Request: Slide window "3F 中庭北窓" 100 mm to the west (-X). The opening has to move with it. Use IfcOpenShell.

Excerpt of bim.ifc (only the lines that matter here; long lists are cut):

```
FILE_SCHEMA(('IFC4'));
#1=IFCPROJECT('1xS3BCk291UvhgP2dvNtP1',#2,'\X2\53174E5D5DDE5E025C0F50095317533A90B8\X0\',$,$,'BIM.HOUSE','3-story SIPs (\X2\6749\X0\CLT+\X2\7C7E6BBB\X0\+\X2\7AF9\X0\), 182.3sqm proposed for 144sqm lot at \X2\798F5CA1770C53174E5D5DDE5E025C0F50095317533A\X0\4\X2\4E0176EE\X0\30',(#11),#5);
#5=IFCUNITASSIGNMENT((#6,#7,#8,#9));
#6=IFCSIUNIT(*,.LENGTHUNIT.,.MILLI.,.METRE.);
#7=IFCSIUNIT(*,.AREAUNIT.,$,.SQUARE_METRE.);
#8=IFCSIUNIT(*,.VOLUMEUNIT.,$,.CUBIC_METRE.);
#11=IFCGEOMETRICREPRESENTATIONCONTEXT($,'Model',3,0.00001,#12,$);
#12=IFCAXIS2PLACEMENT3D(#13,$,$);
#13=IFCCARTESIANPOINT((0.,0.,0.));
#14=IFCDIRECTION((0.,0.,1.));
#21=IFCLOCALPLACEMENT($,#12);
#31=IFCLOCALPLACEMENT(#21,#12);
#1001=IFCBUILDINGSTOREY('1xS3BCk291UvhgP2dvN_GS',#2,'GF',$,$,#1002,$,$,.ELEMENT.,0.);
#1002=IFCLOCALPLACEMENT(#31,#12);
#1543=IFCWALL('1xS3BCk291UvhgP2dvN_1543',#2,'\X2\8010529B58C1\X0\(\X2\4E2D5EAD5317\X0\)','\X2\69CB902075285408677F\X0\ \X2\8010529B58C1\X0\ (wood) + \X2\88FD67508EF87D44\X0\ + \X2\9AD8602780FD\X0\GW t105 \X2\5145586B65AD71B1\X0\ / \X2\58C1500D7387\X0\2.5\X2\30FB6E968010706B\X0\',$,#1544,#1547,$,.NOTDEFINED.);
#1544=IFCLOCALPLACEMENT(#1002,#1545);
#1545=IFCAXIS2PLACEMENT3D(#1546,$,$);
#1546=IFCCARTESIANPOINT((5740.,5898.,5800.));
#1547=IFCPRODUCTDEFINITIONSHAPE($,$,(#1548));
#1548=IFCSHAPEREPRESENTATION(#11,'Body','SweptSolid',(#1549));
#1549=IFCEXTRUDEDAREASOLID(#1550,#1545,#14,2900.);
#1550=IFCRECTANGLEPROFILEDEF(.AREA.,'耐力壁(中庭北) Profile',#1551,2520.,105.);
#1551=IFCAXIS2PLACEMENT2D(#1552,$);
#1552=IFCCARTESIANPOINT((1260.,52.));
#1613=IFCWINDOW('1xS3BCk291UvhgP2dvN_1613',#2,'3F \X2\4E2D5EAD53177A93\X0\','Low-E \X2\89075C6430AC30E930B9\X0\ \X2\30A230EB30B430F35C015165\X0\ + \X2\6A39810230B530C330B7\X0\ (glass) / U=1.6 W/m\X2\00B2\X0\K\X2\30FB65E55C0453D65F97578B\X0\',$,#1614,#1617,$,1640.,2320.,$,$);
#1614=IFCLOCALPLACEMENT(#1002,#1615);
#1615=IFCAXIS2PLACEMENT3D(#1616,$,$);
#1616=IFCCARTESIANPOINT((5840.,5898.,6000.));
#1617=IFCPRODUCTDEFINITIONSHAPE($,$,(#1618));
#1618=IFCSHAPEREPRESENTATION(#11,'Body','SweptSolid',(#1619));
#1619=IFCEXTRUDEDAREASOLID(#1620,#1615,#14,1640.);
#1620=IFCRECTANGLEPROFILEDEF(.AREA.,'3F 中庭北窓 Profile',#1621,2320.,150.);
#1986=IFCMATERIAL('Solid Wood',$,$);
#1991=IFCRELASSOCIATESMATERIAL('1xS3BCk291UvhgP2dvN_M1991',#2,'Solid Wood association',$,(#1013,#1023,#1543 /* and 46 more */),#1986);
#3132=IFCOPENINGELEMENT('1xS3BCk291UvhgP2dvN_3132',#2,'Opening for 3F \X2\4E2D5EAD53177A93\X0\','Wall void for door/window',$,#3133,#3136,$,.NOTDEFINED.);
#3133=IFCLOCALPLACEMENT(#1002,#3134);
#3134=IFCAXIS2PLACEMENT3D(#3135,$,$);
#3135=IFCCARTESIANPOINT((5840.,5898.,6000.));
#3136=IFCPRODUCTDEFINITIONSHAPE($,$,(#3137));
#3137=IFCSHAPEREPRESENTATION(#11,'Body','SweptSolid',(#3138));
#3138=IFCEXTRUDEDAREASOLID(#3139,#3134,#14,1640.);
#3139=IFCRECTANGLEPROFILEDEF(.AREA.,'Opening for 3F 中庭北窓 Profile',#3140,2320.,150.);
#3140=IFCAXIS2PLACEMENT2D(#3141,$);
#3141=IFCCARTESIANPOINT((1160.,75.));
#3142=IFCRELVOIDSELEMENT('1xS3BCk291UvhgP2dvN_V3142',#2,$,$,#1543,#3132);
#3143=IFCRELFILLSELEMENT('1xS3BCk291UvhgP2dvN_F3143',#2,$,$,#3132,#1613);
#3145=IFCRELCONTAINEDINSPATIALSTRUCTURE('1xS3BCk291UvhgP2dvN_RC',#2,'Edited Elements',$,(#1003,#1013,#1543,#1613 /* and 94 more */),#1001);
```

```python
import ifcopenshell
import ifcopenshell.api.geometry
import ifcopenshell.util.placement
import ifcopenshell.util.unit

model = ifcopenshell.open("bim.ifc")
unit_scale = ifcopenshell.util.unit.calculate_unit_scale(model)

window = model.by_guid("1xS3BCk291UvhgP2dvN_1613")
opening = window.FillsVoids[0].RelatingOpeningElement
wall = opening.VoidsElements[0].RelatingBuildingElement

wall_matrix = ifcopenshell.util.placement.get_local_placement(wall.ObjectPlacement)
shift = wall_matrix[:3, 0] * -0.1 / unit_scale
before = ifcopenshell.util.placement.get_local_placement(window.ObjectPlacement)[:3, 3].copy()

# The window is not placed relative to its opening, so move both.
for product in (opening, window):
    matrix = ifcopenshell.util.placement.get_local_placement(product.ObjectPlacement)
    matrix[:3, 3] += shift
    ifcopenshell.api.geometry.edit_object_placement(model, product=product, matrix=matrix, is_si=False)

after = ifcopenshell.util.placement.get_local_placement(window.ObjectPlacement)[:3, 3]
print("window moved by", (after - before).round(3) + 0.0)

model.write("bim_v2.ifc")
```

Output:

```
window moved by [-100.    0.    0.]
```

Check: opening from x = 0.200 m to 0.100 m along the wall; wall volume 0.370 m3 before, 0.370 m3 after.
